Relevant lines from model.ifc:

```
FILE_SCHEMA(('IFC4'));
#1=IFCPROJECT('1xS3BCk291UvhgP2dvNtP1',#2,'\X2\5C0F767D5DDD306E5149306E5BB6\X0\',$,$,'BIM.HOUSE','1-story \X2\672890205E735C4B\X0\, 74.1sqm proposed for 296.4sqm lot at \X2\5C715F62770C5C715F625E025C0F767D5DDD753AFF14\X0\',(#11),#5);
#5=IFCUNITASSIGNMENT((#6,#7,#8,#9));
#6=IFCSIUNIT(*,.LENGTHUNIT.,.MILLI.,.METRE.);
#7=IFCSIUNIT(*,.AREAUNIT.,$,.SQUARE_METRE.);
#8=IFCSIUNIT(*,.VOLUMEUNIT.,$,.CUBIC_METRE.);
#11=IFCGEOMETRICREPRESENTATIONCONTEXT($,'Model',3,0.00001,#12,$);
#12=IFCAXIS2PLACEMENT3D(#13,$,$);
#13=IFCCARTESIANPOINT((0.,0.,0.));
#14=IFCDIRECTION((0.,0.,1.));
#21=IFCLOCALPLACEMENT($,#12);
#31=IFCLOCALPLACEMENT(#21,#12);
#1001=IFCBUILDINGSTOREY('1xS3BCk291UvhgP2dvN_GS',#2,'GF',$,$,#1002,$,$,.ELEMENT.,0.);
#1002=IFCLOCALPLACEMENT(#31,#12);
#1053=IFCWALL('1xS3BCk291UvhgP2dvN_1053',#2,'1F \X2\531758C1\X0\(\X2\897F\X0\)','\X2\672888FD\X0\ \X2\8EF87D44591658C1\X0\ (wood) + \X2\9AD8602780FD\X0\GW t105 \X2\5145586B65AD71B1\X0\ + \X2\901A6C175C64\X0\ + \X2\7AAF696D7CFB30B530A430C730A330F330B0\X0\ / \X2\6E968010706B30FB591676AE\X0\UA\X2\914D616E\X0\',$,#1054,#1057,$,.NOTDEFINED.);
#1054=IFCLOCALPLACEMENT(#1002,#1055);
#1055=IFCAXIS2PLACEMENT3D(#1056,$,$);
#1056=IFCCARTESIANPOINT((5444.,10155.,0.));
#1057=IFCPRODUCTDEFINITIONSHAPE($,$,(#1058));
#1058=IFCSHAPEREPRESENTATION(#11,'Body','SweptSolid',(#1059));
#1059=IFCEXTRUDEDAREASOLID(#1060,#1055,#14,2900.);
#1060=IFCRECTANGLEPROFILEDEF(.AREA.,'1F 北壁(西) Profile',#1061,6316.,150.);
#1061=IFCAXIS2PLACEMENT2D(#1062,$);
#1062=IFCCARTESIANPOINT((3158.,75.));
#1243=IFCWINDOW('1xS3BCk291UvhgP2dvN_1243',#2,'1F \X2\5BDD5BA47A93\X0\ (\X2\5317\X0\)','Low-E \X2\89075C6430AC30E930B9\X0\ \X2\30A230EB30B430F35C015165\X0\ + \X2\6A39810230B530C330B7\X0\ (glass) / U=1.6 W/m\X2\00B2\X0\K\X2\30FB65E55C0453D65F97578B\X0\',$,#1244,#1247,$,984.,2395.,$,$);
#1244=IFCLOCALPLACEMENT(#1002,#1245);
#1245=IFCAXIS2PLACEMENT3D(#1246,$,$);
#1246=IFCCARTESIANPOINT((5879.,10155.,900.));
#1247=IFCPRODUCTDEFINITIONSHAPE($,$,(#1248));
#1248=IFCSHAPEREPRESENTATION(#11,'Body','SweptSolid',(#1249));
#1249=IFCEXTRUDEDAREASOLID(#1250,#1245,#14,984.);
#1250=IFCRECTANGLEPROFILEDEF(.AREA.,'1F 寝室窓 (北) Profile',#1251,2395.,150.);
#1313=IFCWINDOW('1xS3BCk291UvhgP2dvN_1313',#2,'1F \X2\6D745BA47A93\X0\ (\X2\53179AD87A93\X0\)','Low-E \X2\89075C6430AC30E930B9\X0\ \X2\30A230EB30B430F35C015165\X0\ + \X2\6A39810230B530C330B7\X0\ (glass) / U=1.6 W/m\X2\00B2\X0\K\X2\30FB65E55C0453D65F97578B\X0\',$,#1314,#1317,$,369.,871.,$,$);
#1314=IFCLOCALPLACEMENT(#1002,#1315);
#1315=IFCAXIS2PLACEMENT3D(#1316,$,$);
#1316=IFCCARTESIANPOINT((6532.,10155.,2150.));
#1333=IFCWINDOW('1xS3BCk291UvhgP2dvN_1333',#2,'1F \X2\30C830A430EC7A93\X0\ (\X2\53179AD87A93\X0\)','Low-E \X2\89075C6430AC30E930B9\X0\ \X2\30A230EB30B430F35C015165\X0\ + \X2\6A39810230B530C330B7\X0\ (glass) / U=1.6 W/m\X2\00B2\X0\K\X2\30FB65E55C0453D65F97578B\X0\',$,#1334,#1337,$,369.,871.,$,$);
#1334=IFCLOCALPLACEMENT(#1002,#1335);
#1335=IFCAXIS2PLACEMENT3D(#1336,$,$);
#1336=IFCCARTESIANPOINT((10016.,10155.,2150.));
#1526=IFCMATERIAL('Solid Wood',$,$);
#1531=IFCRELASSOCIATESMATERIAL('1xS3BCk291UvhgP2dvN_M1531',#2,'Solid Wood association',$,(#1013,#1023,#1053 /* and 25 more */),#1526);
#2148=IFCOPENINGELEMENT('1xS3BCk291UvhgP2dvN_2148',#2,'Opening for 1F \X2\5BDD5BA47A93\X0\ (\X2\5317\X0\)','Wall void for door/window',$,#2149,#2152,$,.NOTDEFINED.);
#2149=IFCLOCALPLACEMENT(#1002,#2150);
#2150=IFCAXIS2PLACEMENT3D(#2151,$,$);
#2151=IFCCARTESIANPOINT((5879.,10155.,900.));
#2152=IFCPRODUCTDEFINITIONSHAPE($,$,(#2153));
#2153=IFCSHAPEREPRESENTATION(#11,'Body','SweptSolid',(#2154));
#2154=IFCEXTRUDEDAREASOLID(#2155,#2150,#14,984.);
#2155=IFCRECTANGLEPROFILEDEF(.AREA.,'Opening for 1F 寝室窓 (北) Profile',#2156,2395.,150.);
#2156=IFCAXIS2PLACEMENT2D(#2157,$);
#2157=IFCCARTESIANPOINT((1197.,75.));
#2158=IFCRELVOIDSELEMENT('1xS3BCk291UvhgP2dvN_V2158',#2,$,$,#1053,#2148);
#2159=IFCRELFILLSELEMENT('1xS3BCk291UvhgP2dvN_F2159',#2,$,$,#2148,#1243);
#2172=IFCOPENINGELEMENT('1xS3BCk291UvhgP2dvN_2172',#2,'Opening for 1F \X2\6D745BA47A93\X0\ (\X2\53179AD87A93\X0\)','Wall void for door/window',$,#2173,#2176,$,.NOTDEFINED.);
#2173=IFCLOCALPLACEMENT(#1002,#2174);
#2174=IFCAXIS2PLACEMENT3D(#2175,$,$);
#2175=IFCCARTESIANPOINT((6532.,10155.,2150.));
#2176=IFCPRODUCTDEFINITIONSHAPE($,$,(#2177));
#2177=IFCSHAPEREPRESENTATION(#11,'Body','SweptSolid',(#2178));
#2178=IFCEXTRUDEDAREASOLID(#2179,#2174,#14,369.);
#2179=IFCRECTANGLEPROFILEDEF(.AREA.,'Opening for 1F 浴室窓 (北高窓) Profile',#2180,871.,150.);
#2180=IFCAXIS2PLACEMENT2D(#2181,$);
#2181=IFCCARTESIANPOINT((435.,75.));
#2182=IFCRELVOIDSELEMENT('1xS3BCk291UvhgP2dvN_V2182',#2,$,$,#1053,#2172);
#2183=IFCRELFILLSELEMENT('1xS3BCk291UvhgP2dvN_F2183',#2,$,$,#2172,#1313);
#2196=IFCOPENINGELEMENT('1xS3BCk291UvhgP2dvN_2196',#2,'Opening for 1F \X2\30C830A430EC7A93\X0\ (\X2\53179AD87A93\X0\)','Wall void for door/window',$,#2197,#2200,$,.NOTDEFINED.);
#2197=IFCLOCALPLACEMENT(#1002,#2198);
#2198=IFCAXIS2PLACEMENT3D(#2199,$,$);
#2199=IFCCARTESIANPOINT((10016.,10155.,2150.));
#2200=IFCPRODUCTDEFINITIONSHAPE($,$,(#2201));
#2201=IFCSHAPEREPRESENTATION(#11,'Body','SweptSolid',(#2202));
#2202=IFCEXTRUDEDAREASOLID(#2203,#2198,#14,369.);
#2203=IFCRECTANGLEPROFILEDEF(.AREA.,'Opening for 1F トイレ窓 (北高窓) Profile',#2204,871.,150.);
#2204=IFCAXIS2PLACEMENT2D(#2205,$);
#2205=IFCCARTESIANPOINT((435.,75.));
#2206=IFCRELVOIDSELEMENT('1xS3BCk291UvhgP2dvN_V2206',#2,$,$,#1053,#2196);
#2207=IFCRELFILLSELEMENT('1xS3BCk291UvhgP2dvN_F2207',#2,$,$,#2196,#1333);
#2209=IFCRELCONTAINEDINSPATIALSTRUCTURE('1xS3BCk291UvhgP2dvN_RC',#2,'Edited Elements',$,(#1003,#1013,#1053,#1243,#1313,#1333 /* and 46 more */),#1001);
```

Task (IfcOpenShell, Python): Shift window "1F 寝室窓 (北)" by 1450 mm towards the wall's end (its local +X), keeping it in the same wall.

```python
import ifcopenshell
import ifcopenshell.api.geometry
import ifcopenshell.util.placement

model = ifcopenshell.open("model.ifc")

window = model.by_guid("1xS3BCk291UvhgP2dvN_1243")
opening = window.FillsVoids[0].RelatingOpeningElement
wall = opening.VoidsElements[0].RelatingBuildingElement

wall_matrix = ifcopenshell.util.placement.get_local_placement(wall.ObjectPlacement)
shift = wall_matrix[:3, 0] * 1450.0
before = ifcopenshell.util.placement.get_local_placement(window.ObjectPlacement)[:3, 3].copy()

# The window is not placed relative to its opening, so move both.
for product in (opening, window):
    matrix = ifcopenshell.util.placement.get_local_placement(product.ObjectPlacement)
    matrix[:3, 3] += shift
    ifcopenshell.api.geometry.edit_object_placement(model, product=product, matrix=matrix, is_si=False)

after = ifcopenshell.util.placement.get_local_placement(window.ObjectPlacement)[:3, 3]
print("window moved by", (after - before).round(3) + 0.0)

model.write("model_updated.ifc")
```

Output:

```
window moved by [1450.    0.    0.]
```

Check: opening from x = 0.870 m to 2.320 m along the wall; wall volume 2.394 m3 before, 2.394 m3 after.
